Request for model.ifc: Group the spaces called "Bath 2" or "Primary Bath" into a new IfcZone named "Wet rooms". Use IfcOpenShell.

First a look at what the model holds.

```python
import ifcopenshell

model = ifcopenshell.open("model.ifc")
print(model.schema)
seen = {}
for space in model.by_type("IfcSpace"):
    seen[space.LongName] = seen.get(space.LongName, 0) + 1
for name, count in sorted(seen.items(), key=str):
    print(count, "x", name)
print("zones:", [z.Name for z in model.by_type("IfcZone")][:20])
```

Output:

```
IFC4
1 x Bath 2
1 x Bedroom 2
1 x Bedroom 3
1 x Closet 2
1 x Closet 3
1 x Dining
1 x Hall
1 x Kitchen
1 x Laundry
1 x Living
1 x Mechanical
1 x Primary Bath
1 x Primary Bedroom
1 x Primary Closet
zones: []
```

```python
import ifcopenshell
import ifcopenshell.api.group
import ifcopenshell.api.root

model = ifcopenshell.open("model.ifc")

names = {"Bath 2", "Primary Bath"}
spaces = [s for s in model.by_type("IfcSpace") if s.LongName in names]

zone = ifcopenshell.api.root.create_entity(model, ifc_class="IfcZone", name="Wet rooms")
ifcopenshell.api.group.assign_group(model, products=spaces, group=zone)
print(len(spaces), "spaces in", zone.Name)

model.write("model-out.ifc")
```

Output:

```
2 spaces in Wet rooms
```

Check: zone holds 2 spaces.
